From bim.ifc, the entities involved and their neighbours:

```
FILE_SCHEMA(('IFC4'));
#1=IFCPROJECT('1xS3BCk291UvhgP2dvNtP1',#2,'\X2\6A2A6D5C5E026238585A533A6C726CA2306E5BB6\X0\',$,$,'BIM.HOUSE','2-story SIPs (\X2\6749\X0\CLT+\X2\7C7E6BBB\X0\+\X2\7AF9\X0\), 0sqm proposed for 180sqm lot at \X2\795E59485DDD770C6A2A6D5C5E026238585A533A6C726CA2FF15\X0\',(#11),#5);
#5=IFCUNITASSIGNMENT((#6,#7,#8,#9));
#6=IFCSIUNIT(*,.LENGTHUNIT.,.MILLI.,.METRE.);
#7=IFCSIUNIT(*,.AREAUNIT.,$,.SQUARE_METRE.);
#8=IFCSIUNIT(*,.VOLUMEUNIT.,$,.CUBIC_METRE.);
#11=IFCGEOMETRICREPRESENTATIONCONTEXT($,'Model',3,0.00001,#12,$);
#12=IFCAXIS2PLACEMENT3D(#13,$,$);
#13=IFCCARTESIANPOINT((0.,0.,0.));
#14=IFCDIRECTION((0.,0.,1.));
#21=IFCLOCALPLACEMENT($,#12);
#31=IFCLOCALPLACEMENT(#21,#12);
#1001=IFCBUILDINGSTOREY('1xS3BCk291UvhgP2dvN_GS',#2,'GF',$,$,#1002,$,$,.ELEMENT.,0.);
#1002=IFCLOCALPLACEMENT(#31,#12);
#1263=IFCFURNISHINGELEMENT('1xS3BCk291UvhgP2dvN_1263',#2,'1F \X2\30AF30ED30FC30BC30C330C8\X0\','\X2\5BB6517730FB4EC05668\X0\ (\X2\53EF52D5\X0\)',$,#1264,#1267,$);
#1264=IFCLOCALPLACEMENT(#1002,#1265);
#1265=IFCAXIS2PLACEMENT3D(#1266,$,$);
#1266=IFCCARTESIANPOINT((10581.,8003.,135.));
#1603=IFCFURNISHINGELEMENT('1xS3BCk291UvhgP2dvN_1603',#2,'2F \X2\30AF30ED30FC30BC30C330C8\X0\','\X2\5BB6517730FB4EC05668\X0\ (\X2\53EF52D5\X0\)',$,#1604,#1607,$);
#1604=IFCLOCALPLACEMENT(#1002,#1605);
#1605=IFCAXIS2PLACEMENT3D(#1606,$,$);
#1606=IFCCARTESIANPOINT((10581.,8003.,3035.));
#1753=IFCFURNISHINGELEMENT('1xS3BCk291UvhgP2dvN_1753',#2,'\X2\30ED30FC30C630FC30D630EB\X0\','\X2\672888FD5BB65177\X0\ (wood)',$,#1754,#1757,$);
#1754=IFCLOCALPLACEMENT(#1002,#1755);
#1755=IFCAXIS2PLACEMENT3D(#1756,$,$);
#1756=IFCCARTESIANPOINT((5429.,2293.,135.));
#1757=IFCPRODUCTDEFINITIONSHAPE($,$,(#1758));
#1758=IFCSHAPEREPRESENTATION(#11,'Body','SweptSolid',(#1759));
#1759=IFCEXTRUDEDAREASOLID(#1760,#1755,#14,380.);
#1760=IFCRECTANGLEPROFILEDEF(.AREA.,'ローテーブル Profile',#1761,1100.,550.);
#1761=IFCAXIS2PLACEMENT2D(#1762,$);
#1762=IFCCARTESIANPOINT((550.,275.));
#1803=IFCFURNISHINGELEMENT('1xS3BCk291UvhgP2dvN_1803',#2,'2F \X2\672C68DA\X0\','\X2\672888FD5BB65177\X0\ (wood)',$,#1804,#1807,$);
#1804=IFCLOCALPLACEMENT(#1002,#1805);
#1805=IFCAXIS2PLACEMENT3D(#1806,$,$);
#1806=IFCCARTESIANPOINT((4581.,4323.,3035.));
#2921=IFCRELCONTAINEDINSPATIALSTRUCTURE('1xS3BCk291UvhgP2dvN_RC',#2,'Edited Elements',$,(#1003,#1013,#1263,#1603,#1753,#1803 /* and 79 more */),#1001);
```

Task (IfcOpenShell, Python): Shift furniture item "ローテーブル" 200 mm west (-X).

```python
import ifcopenshell
import ifcopenshell.api.geometry
import ifcopenshell.util.placement
import ifcopenshell.util.unit

model = ifcopenshell.open("bim.ifc")
unit_scale = ifcopenshell.util.unit.calculate_unit_scale(model)

item = model.by_id(1753)
matrix = ifcopenshell.util.placement.get_local_placement(item.ObjectPlacement)
matrix[0, 3] -= 0.2 / unit_scale
ifcopenshell.api.geometry.edit_object_placement(model, product=item, matrix=matrix, is_si=False)

print(ifcopenshell.util.placement.get_local_placement(item.ObjectPlacement).round(3) + 0.0)

model.write("bim-out.ifc")
```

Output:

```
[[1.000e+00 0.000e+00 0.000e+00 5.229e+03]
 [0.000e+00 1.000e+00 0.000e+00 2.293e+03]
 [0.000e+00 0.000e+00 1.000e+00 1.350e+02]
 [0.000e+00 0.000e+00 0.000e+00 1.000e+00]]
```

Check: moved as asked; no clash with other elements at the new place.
